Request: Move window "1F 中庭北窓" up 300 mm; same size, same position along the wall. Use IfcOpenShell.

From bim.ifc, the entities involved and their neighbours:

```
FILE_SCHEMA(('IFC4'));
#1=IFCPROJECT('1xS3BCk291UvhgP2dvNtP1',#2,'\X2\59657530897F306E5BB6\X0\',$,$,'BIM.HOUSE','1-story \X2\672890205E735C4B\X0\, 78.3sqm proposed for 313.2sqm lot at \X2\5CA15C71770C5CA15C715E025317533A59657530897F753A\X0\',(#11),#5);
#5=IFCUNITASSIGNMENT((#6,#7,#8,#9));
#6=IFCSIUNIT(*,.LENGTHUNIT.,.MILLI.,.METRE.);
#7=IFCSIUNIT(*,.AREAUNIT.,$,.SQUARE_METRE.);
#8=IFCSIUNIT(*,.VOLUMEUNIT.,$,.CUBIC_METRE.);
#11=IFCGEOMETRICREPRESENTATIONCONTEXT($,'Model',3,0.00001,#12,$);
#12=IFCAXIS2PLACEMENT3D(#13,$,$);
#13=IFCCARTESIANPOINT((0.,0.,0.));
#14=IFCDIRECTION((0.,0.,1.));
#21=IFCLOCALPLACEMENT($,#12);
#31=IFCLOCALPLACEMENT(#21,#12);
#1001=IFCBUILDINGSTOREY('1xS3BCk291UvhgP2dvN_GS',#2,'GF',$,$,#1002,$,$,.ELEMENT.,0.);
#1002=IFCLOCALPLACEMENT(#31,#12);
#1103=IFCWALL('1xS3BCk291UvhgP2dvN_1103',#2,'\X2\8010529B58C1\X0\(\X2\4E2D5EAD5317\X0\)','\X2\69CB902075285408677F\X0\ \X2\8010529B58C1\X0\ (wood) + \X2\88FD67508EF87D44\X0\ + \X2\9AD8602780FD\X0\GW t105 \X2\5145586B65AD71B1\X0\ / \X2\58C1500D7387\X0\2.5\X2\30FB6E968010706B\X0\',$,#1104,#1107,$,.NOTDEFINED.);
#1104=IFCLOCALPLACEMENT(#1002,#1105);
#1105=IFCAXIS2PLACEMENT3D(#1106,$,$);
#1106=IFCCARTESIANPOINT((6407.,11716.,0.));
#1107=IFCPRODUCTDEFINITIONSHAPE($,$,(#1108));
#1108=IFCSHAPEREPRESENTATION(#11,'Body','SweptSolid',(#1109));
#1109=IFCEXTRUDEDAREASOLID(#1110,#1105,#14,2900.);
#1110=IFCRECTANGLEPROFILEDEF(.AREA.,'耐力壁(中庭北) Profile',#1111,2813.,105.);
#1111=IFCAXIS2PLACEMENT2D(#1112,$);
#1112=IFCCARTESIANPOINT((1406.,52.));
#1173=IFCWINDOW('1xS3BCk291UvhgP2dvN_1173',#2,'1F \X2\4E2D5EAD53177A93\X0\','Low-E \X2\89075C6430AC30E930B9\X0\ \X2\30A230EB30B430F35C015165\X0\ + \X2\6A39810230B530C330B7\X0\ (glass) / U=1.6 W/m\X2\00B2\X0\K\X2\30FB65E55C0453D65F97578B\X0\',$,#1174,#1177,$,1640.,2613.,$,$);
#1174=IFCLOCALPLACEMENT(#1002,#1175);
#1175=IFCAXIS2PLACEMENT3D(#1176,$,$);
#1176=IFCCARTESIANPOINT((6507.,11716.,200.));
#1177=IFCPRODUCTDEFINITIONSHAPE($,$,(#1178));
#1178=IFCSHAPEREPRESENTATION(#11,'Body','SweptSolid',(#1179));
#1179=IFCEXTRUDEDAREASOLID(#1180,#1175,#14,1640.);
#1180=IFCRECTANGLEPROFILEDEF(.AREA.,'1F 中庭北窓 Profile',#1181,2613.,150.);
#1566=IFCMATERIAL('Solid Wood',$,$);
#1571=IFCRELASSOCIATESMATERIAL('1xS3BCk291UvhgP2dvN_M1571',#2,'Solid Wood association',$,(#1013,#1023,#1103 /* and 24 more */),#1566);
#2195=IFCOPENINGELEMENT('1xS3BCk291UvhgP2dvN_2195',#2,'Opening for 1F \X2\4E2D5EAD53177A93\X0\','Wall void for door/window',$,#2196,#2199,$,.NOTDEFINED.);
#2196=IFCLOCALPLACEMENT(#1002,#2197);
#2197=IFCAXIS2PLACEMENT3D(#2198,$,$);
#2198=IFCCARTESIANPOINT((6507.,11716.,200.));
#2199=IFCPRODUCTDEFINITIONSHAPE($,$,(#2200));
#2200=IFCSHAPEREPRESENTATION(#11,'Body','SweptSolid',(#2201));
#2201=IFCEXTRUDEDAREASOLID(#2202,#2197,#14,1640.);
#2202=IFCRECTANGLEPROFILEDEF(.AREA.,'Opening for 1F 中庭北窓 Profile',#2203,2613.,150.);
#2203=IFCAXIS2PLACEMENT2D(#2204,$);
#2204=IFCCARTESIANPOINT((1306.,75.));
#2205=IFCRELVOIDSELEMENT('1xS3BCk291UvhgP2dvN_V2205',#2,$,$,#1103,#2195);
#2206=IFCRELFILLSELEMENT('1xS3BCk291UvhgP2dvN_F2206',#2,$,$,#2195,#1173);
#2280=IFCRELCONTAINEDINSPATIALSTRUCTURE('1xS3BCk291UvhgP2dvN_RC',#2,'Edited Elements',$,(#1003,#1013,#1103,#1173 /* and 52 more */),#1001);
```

```python
import numpy as np
import ifcopenshell
import ifcopenshell.api.geometry
import ifcopenshell.util.placement
import ifcopenshell.util.unit

model = ifcopenshell.open("bim.ifc")
unit_scale = ifcopenshell.util.unit.calculate_unit_scale(model)

window = model.by_guid("1xS3BCk291UvhgP2dvN_1173")
opening = window.FillsVoids[0].RelatingOpeningElement
dz = 300.0

shift = np.array([0.0, 0.0, dz])
# The window is not placed relative to its opening, so move both.
for product in (opening, window):
    matrix = ifcopenshell.util.placement.get_local_placement(product.ObjectPlacement)
    matrix[:3, 3] += shift
    ifcopenshell.api.geometry.edit_object_placement(model, product=product, matrix=matrix, is_si=False)

print(f"moved by {dz * unit_scale:+.3f} m")

model.write("bim-out.ifc")
```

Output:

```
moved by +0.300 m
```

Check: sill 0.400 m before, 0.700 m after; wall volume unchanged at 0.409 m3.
